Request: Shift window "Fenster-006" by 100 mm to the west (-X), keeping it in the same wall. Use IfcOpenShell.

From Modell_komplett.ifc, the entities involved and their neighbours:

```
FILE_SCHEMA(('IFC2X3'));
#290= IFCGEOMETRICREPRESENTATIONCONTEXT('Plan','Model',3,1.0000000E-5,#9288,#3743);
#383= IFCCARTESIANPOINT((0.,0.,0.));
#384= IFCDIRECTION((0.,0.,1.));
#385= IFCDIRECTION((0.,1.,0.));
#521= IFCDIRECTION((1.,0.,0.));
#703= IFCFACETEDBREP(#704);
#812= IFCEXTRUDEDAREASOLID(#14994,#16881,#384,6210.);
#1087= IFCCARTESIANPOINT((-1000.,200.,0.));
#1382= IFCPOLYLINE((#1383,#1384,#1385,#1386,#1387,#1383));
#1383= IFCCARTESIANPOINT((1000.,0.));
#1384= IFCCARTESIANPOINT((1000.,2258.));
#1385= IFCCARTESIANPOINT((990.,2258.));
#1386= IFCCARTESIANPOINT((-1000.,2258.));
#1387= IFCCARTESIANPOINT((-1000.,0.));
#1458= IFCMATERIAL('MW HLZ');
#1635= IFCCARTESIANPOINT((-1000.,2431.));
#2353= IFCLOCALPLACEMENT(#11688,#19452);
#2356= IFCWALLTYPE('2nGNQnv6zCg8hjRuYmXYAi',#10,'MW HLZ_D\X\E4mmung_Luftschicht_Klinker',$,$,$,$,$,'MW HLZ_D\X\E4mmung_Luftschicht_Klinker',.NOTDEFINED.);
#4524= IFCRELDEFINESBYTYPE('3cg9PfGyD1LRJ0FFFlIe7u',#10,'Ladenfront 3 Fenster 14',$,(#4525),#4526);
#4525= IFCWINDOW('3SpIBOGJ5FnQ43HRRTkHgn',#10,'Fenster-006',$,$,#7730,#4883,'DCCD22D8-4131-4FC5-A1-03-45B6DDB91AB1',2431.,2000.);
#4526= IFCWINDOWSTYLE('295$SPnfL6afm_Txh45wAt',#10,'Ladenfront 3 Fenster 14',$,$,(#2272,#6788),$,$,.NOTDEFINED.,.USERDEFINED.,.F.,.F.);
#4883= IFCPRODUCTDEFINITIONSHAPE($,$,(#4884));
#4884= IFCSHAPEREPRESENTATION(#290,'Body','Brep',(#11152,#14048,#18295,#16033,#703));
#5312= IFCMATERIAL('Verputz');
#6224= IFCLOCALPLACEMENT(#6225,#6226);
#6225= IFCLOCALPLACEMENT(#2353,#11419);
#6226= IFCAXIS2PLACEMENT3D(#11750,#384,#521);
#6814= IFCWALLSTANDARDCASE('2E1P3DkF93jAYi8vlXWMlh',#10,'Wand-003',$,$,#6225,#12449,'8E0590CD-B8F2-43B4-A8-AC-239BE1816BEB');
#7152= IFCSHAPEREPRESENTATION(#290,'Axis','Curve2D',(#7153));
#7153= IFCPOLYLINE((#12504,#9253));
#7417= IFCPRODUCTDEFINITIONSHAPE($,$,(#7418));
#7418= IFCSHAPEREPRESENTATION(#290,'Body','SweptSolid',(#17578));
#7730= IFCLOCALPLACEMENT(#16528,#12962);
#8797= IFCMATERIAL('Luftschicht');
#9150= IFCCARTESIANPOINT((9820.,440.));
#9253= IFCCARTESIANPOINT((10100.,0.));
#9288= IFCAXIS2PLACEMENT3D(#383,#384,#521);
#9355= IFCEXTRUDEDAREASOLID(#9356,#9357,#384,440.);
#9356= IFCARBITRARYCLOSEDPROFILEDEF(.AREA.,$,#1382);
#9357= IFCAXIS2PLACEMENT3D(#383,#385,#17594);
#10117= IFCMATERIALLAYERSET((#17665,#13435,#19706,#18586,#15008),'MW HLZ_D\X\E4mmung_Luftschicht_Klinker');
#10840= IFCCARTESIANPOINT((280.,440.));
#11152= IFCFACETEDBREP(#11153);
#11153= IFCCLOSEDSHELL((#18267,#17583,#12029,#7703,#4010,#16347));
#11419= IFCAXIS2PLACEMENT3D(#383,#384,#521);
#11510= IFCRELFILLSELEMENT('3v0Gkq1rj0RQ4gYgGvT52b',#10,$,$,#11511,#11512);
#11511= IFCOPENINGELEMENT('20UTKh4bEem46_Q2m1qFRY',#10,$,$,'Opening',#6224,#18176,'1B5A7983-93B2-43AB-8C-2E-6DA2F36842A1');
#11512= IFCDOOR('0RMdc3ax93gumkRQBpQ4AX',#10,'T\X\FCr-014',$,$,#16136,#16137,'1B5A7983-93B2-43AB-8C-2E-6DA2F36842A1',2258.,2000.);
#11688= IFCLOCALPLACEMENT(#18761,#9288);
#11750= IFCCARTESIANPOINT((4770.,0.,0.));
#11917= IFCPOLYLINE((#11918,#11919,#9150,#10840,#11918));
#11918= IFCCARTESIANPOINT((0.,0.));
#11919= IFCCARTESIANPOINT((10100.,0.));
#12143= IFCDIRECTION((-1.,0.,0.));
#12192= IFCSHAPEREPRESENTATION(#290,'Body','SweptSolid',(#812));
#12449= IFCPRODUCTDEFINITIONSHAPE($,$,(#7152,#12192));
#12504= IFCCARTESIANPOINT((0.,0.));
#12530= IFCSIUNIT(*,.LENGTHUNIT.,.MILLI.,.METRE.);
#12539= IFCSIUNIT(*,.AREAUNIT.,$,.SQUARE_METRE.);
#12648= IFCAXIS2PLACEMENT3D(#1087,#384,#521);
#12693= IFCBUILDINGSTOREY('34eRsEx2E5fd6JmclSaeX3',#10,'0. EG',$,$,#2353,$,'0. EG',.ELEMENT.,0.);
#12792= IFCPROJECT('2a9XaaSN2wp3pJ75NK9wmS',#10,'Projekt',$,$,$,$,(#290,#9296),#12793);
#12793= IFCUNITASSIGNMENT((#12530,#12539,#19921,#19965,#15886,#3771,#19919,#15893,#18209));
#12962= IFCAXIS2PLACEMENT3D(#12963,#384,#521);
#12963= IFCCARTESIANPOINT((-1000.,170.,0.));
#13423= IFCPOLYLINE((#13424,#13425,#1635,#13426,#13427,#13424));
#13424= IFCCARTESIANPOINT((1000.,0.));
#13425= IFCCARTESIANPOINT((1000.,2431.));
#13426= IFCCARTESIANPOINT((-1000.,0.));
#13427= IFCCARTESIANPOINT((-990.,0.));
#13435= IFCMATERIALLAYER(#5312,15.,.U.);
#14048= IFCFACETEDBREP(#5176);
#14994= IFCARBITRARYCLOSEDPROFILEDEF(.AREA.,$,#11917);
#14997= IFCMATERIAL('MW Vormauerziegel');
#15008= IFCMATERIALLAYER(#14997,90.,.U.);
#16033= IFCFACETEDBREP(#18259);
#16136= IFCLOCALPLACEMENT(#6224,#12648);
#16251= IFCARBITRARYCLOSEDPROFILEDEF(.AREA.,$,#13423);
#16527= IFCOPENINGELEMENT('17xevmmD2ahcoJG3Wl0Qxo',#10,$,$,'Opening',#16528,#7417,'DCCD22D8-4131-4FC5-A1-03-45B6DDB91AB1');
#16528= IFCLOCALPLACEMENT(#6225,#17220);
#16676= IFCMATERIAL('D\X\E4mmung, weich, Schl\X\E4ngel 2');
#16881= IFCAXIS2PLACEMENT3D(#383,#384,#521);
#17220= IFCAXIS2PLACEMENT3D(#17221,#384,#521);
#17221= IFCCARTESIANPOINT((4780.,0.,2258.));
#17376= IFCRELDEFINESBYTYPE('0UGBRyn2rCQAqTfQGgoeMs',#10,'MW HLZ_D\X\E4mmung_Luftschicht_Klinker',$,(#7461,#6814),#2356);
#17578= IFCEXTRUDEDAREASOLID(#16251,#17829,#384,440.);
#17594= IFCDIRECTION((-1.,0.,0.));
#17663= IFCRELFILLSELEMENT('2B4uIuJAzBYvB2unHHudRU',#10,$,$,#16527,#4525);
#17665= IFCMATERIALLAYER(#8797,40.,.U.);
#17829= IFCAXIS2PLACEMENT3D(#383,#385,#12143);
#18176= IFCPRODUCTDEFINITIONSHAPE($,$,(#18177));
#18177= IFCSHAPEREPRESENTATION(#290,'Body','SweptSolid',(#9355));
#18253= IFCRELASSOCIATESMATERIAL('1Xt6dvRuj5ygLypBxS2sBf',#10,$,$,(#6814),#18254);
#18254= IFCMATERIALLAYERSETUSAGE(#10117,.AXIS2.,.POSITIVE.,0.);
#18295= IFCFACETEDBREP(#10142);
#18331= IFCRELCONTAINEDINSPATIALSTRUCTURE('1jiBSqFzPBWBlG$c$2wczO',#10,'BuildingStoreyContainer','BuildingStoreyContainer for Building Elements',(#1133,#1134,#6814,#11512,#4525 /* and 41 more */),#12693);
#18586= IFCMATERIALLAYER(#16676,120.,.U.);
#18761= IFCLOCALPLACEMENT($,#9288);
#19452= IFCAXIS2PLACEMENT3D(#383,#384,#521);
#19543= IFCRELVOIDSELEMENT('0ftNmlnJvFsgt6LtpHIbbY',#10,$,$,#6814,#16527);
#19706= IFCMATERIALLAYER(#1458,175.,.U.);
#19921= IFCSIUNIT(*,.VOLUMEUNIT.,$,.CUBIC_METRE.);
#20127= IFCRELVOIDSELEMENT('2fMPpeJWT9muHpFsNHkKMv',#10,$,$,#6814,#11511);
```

```python
import ifcopenshell
import ifcopenshell.api.geometry
import ifcopenshell.util.placement
import ifcopenshell.util.unit

model = ifcopenshell.open("Modell_komplett.ifc")
unit_scale = ifcopenshell.util.unit.calculate_unit_scale(model)

window = model.by_id(4525)
opening = window.FillsVoids[0].RelatingOpeningElement
wall = opening.VoidsElements[0].RelatingBuildingElement

wall_matrix = ifcopenshell.util.placement.get_local_placement(wall.ObjectPlacement)
shift = wall_matrix[:3, 0] * -0.1 / unit_scale
before = ifcopenshell.util.placement.get_local_placement(window.ObjectPlacement)[:3, 3].copy()

# The window is placed relative to its opening, so it follows when the opening moves.
matrix = ifcopenshell.util.placement.get_local_placement(opening.ObjectPlacement)
matrix[:3, 3] += shift
ifcopenshell.api.geometry.edit_object_placement(
    model, product=opening, matrix=matrix, is_si=False, should_transform_children=True
)

after = ifcopenshell.util.placement.get_local_placement(window.ObjectPlacement)[:3, 3]
print("window moved by", (after - before).round(3) + 0.0)

model.write("Modell_komplett-out.ifc")
```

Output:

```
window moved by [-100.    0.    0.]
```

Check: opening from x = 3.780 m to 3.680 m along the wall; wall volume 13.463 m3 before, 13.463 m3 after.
